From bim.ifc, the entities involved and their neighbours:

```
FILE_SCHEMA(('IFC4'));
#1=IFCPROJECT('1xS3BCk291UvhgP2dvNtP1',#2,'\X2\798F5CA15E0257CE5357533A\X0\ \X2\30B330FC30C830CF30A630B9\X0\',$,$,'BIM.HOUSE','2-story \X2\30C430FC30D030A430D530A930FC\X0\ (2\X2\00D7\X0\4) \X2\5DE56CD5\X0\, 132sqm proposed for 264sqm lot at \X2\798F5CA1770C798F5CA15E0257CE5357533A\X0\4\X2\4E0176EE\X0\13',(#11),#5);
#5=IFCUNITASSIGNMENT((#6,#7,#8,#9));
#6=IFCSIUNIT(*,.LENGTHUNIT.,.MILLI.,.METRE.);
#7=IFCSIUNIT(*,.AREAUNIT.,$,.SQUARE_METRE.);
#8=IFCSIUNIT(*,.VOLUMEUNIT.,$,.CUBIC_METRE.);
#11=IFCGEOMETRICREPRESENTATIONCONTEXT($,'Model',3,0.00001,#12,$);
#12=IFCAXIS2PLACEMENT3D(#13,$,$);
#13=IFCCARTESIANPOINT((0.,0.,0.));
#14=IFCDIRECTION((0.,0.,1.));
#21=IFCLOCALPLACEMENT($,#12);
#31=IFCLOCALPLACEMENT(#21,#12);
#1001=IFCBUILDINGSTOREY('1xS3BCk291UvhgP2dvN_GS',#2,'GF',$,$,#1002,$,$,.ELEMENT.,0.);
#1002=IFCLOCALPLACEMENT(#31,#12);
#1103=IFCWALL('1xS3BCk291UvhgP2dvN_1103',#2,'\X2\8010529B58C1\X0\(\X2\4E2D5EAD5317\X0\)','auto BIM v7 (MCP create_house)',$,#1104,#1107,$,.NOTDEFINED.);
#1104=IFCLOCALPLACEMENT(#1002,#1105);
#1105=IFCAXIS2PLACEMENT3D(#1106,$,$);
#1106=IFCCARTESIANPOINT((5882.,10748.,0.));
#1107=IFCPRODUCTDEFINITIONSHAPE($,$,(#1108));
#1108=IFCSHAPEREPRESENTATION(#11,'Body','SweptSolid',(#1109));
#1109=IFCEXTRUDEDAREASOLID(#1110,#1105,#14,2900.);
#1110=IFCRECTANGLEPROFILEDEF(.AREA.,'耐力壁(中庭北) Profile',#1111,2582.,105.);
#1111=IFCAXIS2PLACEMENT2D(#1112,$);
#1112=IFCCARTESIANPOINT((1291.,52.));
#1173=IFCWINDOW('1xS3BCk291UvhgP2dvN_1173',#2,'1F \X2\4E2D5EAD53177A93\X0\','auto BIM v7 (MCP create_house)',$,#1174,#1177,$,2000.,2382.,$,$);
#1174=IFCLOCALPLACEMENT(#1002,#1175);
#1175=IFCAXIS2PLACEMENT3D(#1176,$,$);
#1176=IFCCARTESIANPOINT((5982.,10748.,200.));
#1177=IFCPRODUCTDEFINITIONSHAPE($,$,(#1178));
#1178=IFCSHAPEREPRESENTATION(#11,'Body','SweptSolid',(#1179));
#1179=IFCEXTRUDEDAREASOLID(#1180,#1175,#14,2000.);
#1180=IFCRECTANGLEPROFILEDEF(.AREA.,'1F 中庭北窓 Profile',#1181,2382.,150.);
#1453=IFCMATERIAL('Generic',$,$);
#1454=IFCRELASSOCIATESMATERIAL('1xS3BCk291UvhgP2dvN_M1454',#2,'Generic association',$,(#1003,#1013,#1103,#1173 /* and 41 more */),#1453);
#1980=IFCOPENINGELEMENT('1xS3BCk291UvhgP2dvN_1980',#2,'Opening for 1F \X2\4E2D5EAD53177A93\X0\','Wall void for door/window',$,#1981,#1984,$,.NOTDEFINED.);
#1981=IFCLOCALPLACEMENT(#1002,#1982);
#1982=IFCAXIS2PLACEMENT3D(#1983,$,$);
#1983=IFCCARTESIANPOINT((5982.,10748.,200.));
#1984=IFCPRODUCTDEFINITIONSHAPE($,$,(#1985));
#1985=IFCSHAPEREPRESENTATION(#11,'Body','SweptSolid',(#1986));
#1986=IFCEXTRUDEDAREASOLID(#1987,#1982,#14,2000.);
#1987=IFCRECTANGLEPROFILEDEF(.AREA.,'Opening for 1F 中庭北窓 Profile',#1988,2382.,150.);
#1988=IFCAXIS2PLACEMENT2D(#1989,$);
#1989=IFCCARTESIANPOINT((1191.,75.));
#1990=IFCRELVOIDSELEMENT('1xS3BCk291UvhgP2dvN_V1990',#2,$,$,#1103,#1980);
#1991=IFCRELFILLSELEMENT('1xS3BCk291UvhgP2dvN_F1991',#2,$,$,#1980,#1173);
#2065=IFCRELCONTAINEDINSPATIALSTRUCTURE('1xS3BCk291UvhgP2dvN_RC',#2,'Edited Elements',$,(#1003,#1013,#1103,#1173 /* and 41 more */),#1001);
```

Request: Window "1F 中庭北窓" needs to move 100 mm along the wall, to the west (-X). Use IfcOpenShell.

```python
import ifcopenshell
import ifcopenshell.api.geometry
import ifcopenshell.util.placement
import ifcopenshell.util.unit

model = ifcopenshell.open("bim.ifc")
unit_scale = ifcopenshell.util.unit.calculate_unit_scale(model)

window = model.by_guid("1xS3BCk291UvhgP2dvN_1173")
opening = window.FillsVoids[0].RelatingOpeningElement
wall = opening.VoidsElements[0].RelatingBuildingElement

wall_matrix = ifcopenshell.util.placement.get_local_placement(wall.ObjectPlacement)
shift = wall_matrix[:3, 0] * -0.1 / unit_scale
before = ifcopenshell.util.placement.get_local_placement(window.ObjectPlacement)[:3, 3].copy()

# The window is not placed relative to its opening, so move both.
for product in (opening, window):
    matrix = ifcopenshell.util.placement.get_local_placement(product.ObjectPlacement)
    matrix[:3, 3] += shift
    ifcopenshell.api.geometry.edit_object_placement(model, product=product, matrix=matrix, is_si=False)

after = ifcopenshell.util.placement.get_local_placement(window.ObjectPlacement)[:3, 3]
print("window moved by", (after - before).round(3) + 0.0)

model.write("bim_v2.ifc")
```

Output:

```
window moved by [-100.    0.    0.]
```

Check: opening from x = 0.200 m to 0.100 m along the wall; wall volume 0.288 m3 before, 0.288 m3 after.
